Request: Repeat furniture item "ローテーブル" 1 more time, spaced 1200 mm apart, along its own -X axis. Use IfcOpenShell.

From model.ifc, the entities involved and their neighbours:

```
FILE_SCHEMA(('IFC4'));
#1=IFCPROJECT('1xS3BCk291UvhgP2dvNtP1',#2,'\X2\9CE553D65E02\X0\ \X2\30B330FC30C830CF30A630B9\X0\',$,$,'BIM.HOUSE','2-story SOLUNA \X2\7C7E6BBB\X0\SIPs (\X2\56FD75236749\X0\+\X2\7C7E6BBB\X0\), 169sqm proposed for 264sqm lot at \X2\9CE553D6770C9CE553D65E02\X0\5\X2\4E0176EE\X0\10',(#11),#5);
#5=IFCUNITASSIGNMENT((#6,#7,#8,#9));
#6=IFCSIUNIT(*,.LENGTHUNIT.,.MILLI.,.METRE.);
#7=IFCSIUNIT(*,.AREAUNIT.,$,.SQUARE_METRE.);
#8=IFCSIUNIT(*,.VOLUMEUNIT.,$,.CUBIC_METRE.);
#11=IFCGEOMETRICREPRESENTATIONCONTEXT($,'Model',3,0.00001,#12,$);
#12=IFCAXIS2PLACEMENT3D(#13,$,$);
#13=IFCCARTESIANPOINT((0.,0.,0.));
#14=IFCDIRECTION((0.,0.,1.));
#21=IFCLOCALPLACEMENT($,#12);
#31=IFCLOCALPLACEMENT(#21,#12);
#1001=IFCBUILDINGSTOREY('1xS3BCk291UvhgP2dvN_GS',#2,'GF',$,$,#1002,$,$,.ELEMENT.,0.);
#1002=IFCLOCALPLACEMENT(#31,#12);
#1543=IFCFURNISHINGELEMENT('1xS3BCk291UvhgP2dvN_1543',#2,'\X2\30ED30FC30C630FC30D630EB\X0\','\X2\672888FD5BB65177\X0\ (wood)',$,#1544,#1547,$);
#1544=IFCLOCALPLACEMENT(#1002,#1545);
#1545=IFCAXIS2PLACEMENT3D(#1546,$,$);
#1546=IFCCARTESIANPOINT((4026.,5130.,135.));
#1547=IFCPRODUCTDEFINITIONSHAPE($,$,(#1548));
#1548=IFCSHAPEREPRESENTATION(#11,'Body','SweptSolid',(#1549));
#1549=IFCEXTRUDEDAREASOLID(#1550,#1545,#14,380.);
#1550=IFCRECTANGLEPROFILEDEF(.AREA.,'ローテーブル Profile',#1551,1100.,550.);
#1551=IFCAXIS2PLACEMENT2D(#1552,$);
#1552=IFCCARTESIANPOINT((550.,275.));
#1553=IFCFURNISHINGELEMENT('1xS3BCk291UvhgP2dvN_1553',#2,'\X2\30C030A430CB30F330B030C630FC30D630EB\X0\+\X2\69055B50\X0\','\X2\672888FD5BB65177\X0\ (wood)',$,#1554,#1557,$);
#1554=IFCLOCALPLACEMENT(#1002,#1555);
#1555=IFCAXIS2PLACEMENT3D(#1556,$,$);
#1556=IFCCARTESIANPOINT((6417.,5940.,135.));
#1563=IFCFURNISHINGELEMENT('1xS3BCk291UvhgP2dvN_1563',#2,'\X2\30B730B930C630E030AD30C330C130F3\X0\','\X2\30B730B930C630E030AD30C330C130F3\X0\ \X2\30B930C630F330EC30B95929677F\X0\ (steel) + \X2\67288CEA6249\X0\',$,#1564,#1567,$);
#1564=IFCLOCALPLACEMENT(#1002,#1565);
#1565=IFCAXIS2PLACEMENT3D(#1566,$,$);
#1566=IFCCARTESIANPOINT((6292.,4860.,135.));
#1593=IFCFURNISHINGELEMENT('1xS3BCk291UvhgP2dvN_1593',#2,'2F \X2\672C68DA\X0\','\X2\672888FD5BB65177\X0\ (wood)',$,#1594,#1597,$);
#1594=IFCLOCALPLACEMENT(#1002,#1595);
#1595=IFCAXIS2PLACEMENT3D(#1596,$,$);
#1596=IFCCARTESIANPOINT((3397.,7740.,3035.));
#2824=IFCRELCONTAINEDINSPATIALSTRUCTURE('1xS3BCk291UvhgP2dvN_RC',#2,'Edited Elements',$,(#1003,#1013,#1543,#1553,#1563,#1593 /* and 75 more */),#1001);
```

```python
import ifcopenshell
import ifcopenshell.api.geometry
import ifcopenshell.api.root
import ifcopenshell.util.element
import ifcopenshell.util.placement

model = ifcopenshell.open("model.ifc")


def reuse_history(source, copy):
    """copy_class also copies each property set's owner history, people and application; keep the originals."""
    for rel in copy.IsDefinedBy:
        if rel.is_a("IfcRelDefinesByProperties") and (history := rel.RelatingPropertyDefinition.OwnerHistory):
            rel.RelatingPropertyDefinition.OwnerHistory = source.OwnerHistory
            ifcopenshell.util.element.remove_deep2(model, history)


source = model.by_guid("1xS3BCk291UvhgP2dvN_1543")
base = ifcopenshell.util.placement.get_local_placement(source.ObjectPlacement)
step = -base[:3, 0] * 1200.0

for i in range(1, 2):
    copy = ifcopenshell.api.root.copy_class(model, product=source)
    copy.Representation = ifcopenshell.util.element.copy_deep(
        model, source.Representation, exclude=["IfcGeometricRepresentationContext", "IfcRepresentationMap"]
    )
    reuse_history(source, copy)
    matrix = base.copy()
    matrix[:3, 3] += i * step
    print("added at", matrix[:3, 3].round(3) + 0.0)
    ifcopenshell.api.geometry.edit_object_placement(model, product=copy, matrix=matrix, is_si=False)

model.write("model-out.ifc")
```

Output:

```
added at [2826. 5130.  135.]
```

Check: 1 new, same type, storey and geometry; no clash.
